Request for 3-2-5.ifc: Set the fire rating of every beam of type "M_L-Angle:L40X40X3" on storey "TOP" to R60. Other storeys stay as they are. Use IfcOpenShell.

First a look at what the model holds.

```python
import ifcopenshell
import ifcopenshell.util.element

model = ifcopenshell.open("3-2-5.ifc")
print(model.schema)
storey = next(s for s in model.by_type("IfcBuildingStorey") if s.Name == "TOP")
beams = [e for e in ifcopenshell.util.element.get_decomposition(storey) if e.is_a("IfcBeam")]
seen = {}
for e in beams:
    element_type = ifcopenshell.util.element.get_type(e)
    key = (element_type.Name if element_type != e and element_type else None, ifcopenshell.util.element.get_pset(e, "Pset_BeamCommon", "FireRating"))
    seen[key] = seen.get(key, 0) + 1
for (name, value), count in sorted(seen.items(), key=str):
    print(count, "x", name, "|", value)
```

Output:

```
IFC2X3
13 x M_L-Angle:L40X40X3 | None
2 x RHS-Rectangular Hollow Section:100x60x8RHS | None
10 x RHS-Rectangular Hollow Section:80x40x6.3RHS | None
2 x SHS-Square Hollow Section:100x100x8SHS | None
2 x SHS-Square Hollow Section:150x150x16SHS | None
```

```python
import ifcopenshell
import ifcopenshell.api.pset
import ifcopenshell.util.element

model = ifcopenshell.open("3-2-5.ifc")

storey = next(s for s in model.by_type("IfcBuildingStorey") if s.Name == "TOP")
beams = [e for e in ifcopenshell.util.element.get_decomposition(storey) if e.is_a("IfcBeam")]

count = 0
for e in beams:
    element_type = ifcopenshell.util.element.get_type(e)
    if element_type in (None, e) or element_type.Name != "M_L-Angle:L40X40X3":
        continue
    # add_pset returns the element's existing set when there is one.
    pset = ifcopenshell.api.pset.add_pset(model, product=e, name="Pset_BeamCommon")
    ifcopenshell.api.pset.edit_pset(model, pset=pset, properties={"FireRating": "R60"})
    count += 1

print(count, "beams updated")

model.write("3-2-5_v2.ifc")
```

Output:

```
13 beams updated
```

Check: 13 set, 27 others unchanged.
